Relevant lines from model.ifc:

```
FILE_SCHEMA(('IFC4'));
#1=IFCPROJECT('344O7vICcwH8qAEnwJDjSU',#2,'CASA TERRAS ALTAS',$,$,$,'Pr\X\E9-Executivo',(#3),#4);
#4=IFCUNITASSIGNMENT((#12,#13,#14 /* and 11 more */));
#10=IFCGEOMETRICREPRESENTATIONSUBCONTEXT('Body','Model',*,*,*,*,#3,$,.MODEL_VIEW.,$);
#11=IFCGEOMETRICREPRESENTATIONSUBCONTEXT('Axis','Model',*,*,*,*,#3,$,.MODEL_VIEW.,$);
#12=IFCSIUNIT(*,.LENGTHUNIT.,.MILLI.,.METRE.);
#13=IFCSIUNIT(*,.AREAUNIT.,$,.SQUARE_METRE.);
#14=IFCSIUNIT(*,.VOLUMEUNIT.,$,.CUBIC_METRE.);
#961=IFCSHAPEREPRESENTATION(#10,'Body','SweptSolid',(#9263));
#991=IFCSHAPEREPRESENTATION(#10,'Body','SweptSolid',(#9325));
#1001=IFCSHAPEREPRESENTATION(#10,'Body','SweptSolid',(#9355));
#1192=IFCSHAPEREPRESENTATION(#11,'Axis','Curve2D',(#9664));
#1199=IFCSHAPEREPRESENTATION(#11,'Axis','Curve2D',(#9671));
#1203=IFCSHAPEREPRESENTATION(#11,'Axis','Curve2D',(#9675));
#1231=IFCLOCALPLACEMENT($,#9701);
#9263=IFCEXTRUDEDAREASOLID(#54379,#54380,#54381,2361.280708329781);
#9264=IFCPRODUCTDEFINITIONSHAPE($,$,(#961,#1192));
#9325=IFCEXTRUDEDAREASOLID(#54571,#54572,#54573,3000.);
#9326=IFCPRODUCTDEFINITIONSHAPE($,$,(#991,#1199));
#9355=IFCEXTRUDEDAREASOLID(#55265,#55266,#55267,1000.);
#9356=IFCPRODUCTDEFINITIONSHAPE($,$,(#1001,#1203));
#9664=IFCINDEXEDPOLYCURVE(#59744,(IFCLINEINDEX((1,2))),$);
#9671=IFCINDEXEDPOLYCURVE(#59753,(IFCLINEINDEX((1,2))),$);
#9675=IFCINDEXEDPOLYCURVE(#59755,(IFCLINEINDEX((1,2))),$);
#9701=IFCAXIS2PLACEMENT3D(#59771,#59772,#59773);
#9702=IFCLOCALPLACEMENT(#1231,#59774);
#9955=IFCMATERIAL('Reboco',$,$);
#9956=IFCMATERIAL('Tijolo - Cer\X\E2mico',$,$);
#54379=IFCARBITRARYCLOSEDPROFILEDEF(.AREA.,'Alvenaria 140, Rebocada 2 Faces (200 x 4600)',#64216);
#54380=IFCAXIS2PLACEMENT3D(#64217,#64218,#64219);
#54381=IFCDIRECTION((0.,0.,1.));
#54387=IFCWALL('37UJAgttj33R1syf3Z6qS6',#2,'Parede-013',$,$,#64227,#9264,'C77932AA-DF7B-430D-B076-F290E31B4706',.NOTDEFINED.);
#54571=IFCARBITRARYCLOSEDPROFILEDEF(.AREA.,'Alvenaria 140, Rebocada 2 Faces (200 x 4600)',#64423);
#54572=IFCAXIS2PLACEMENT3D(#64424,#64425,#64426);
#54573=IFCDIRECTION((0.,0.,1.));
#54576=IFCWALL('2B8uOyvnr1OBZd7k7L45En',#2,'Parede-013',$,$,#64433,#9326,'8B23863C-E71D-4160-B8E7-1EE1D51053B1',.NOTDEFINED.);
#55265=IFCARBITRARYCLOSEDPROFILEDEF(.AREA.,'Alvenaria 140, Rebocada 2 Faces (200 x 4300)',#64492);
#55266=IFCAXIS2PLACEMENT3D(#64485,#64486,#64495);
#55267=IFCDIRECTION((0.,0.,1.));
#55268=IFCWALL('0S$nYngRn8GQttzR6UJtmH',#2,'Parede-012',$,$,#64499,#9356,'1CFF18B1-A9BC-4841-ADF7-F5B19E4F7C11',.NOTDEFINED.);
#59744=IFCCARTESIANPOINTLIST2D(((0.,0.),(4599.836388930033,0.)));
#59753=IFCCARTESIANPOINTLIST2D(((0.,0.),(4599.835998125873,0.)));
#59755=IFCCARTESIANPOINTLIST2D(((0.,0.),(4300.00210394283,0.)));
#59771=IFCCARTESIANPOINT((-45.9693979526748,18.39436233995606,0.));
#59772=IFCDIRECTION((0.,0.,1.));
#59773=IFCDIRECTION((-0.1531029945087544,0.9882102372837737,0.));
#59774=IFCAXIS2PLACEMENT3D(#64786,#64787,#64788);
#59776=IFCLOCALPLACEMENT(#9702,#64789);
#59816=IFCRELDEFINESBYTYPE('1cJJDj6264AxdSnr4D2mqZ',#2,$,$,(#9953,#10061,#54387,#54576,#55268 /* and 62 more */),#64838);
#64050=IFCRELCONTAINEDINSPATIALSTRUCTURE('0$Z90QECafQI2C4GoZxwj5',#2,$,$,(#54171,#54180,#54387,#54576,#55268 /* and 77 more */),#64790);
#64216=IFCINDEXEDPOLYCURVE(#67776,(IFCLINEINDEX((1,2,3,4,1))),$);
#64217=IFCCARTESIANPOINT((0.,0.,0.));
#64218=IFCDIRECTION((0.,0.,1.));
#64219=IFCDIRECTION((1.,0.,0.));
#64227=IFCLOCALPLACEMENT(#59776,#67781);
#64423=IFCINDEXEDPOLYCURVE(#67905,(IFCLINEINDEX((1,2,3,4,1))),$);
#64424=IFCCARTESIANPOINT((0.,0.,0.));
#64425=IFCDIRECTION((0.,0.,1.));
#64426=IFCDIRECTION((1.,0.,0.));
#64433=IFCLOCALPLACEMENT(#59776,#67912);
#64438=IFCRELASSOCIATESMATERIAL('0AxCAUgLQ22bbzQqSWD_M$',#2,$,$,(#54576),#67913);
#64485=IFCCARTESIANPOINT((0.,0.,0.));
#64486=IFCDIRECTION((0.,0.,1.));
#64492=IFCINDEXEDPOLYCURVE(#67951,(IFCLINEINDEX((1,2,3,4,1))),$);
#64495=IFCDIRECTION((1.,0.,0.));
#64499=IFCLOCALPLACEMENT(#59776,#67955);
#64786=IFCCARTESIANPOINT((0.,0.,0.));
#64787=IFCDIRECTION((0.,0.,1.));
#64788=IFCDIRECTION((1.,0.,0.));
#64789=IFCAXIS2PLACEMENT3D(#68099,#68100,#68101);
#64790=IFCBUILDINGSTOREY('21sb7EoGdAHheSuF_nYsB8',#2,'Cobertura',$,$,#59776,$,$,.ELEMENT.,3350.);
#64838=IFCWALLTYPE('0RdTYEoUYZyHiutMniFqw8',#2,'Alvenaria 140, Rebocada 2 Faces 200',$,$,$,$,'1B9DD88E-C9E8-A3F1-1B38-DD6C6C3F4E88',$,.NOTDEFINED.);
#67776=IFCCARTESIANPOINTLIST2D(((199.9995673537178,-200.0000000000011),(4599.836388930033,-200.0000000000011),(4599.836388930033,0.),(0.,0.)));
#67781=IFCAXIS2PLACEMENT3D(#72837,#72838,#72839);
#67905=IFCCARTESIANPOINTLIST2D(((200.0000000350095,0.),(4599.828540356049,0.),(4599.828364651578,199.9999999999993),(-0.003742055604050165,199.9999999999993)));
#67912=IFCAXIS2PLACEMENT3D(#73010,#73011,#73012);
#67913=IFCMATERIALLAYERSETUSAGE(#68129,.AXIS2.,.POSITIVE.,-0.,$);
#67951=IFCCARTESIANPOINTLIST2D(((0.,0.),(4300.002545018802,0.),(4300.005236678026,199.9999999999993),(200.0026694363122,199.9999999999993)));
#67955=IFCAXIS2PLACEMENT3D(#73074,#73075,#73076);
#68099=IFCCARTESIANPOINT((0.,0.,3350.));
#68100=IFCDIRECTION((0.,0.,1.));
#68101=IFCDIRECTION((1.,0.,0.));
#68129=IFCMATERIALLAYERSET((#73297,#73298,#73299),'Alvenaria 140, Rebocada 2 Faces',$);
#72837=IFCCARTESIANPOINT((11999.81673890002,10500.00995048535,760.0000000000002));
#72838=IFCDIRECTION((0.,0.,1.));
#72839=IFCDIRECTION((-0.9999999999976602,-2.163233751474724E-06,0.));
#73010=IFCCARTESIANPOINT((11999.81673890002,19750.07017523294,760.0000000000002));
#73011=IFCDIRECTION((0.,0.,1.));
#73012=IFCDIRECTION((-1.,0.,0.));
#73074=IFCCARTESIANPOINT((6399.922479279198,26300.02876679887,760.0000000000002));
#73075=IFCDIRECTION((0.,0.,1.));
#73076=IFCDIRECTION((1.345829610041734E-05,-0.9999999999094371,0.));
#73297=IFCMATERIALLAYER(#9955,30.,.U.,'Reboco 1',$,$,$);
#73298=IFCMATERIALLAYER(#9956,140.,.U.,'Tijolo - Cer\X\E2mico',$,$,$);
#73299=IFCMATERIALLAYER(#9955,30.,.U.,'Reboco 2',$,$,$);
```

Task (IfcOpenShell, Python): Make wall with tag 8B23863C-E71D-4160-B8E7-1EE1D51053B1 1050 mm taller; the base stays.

```python
import ifcopenshell
import ifcopenshell.geom
import ifcopenshell.util.representation
import ifcopenshell.util.shape
import ifcopenshell.util.unit

model = ifcopenshell.open("model.ifc")
unit_scale = ifcopenshell.util.unit.calculate_unit_scale(model)
settings = ifcopenshell.geom.settings()


def volume(element):
    """Net volume in cubic metres, openings subtracted."""
    shape = ifcopenshell.geom.create_shape(settings, element)
    return ifcopenshell.util.shape.get_volume(shape.geometry)


wall = model.by_guid("2B8uOyvnr1OBZd7k7L45En")
before = volume(wall)

body = ifcopenshell.util.representation.get_representation(wall, "Model", "Body")
solid = body.Items[0]
old_height = solid.Depth
solid.Depth += 1.05 / unit_scale
after = volume(wall)

print(f"height {old_height:g} -> {solid.Depth:g}, volume {before:.3f} -> {after:.3f} m3")

model.write("model-out.ifc")
```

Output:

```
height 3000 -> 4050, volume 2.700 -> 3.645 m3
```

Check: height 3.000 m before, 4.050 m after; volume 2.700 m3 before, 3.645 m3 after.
